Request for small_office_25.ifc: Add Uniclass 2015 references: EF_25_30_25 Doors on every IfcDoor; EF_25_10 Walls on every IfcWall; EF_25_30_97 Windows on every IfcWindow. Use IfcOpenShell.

First a look at what the model holds.

```python
import ifcopenshell

model = ifcopenshell.open("small_office_25.ifc")
print(model.schema)
print("classifications:", [c.Name for c in model.by_type("IfcClassification")])
for ifc_class in ("IfcDoor", "IfcRoof", "IfcStair", "IfcWall", "IfcWindow"):
    print(ifc_class, len(model.by_type(ifc_class)))
```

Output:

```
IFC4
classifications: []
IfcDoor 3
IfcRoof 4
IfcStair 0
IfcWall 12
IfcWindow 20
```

```python
import ifcopenshell
import ifcopenshell.api.classification

model = ifcopenshell.open("small_office_25.ifc")

system = ifcopenshell.api.classification.add_classification(model, classification="Uniclass 2015")

codes = {
    "IfcDoor": ("EF_25_30_25", "Doors"),
    "IfcWall": ("EF_25_10", "Walls"),
    "IfcWindow": ("EF_25_30_97", "Windows"),
}
for ifc_class, (code, name) in codes.items():
    products = model.by_type(ifc_class)
    ifcopenshell.api.classification.add_reference(
        model, products=products, classification=system, identification=code, name=name
    )
    print(code, len(products))

model.write("small_office_25_rev.ifc")
```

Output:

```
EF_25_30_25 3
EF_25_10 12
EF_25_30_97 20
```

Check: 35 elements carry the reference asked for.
